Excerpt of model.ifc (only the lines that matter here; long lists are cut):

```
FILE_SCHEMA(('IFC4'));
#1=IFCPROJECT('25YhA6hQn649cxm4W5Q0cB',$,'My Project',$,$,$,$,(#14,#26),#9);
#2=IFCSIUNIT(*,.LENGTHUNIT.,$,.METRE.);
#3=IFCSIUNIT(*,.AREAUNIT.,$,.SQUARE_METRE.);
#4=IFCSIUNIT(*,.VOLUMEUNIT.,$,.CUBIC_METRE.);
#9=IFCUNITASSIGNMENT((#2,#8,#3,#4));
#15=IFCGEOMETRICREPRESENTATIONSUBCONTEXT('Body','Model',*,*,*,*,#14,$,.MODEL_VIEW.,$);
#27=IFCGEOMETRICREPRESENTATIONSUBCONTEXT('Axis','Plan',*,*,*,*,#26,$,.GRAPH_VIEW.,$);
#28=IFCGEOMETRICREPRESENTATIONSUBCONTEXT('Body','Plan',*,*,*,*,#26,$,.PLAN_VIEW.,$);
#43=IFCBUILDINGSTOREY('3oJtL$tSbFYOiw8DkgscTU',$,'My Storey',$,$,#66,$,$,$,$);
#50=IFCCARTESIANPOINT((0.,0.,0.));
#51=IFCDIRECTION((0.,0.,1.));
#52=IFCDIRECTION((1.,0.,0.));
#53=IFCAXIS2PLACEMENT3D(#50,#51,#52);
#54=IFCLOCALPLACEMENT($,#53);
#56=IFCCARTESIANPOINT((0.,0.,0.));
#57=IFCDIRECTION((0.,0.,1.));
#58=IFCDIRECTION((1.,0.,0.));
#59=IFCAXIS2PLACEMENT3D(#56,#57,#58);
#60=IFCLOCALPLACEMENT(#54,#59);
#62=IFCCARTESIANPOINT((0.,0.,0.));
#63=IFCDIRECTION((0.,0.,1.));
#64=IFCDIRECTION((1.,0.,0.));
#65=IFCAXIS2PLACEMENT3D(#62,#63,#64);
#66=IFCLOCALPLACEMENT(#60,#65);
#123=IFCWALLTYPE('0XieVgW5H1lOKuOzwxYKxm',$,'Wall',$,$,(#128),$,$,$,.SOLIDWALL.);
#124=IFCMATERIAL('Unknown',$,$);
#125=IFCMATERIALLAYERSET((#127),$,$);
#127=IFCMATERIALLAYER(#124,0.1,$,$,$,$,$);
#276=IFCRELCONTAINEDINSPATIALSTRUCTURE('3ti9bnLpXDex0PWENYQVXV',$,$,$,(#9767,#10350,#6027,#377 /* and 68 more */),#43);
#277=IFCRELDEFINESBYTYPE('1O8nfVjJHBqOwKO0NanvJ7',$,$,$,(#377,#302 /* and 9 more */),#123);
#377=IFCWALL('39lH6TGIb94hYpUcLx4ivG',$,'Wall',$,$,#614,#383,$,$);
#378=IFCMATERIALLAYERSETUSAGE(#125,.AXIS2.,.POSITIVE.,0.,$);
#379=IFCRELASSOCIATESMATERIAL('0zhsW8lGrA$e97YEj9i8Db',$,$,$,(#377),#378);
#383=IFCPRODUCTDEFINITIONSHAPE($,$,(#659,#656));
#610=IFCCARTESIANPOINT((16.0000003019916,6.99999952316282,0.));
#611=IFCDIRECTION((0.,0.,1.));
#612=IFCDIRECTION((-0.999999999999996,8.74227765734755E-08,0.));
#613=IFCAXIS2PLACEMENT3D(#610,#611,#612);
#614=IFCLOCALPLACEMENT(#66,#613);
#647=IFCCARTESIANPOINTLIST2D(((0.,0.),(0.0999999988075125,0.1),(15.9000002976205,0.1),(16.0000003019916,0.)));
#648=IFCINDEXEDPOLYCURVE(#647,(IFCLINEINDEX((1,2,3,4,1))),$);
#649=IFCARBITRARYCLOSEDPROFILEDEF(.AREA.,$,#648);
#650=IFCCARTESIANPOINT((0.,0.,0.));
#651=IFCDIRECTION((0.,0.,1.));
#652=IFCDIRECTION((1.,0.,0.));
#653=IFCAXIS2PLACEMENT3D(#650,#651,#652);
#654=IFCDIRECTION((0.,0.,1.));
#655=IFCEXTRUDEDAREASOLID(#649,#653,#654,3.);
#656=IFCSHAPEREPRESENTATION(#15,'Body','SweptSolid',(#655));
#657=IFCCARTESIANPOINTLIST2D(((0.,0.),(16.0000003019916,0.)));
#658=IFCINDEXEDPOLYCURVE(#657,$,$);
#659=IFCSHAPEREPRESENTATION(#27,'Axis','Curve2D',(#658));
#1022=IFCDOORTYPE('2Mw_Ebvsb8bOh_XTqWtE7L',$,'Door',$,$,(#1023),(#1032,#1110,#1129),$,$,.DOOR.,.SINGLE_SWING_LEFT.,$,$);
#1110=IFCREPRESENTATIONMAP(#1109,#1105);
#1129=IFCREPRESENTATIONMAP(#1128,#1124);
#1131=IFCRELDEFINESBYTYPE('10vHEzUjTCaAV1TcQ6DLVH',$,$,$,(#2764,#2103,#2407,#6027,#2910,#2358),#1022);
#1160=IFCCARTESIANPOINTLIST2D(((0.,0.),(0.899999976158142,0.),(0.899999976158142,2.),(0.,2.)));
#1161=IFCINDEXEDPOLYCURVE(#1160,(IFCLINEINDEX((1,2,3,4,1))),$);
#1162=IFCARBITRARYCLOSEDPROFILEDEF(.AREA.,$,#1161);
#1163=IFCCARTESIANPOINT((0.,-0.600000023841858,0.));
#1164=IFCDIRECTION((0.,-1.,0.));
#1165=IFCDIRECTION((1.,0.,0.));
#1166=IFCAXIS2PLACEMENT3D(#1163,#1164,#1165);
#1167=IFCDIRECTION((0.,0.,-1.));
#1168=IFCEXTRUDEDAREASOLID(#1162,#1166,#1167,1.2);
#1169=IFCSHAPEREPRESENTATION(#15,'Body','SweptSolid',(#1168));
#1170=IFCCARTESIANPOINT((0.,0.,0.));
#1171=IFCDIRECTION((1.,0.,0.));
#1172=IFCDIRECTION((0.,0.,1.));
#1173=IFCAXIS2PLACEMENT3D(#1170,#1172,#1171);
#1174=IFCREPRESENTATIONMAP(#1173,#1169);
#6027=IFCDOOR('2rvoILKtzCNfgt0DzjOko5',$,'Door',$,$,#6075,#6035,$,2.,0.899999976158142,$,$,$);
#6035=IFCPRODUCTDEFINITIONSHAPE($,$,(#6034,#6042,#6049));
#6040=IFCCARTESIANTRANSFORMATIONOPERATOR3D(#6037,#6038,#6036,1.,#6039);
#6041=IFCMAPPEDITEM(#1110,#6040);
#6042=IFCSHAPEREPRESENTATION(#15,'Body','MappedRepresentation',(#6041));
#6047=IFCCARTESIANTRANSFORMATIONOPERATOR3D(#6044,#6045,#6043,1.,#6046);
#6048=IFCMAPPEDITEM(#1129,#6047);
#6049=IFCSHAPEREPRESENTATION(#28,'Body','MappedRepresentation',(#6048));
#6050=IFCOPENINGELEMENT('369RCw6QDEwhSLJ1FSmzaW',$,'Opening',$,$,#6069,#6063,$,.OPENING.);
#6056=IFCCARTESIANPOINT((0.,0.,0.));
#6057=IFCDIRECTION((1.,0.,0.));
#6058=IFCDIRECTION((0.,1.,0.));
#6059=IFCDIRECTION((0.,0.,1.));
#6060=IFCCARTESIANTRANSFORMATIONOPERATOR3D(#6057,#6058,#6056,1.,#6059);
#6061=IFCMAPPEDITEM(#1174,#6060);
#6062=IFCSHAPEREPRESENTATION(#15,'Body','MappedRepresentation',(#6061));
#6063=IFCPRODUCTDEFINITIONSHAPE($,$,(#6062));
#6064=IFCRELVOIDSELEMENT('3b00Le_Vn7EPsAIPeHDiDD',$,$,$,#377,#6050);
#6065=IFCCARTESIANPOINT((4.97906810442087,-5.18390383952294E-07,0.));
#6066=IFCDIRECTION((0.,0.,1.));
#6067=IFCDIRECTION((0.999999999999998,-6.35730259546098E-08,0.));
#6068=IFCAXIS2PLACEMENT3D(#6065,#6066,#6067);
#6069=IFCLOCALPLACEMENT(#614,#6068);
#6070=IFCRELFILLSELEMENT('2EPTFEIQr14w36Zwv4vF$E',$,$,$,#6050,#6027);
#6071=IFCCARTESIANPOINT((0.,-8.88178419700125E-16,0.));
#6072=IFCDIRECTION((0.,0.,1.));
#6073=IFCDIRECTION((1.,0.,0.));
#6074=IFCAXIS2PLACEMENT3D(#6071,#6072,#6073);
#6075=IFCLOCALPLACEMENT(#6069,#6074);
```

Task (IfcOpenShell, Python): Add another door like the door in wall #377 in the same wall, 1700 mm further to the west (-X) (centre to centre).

```python
import ifcopenshell
import ifcopenshell.api.feature
import ifcopenshell.api.geometry
import ifcopenshell.api.root
import ifcopenshell.geom
import ifcopenshell.util.element
import ifcopenshell.util.placement
import ifcopenshell.util.shape

model = ifcopenshell.open("model.ifc")
settings = ifcopenshell.geom.settings()


def volume(element):
    """Net volume in cubic metres, openings subtracted."""
    shape = ifcopenshell.geom.create_shape(settings, element)
    return ifcopenshell.util.shape.get_volume(shape.geometry)


door = model.by_id(6027)
opening = door.FillsVoids[0].RelatingOpeningElement
wall = opening.VoidsElements[0].RelatingBuildingElement
before = volume(wall)
shift = ifcopenshell.util.placement.get_local_placement(wall.ObjectPlacement)[:3, 0] * 1.7

# copy_class copies the void relationship, type, container and properties, but no geometry.
new_opening = ifcopenshell.api.root.copy_class(model, product=opening)
new_opening.Representation = ifcopenshell.util.element.copy_deep(
    model, opening.Representation, exclude=["IfcGeometricRepresentationContext", "IfcRepresentationMap"]
)
new_door = ifcopenshell.api.root.copy_class(model, product=door)
new_door.Representation = ifcopenshell.util.element.copy_deep(
    model, door.Representation, exclude=["IfcGeometricRepresentationContext", "IfcRepresentationMap"]
)
ifcopenshell.api.feature.add_filling(model, opening=new_opening, element=new_door)

for old, new in ((opening, new_opening), (door, new_door)):
    matrix = ifcopenshell.util.placement.get_local_placement(old.ObjectPlacement)
    matrix[:3, 3] += shift
    ifcopenshell.api.geometry.edit_object_placement(model, product=new, matrix=matrix, is_si=False)

after = volume(wall)

print(f"wall volume {before:.3f} -> {after:.3f} m3")

model.write("model_rev.ifc")
```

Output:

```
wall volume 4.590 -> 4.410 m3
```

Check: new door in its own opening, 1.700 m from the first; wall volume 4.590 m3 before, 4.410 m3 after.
